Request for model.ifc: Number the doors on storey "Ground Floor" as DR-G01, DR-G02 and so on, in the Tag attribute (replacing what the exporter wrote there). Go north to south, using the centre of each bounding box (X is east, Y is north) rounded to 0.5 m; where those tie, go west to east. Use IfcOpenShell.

First a look at what the model holds.

```python
import ifcopenshell
import ifcopenshell.util.element
import ifcopenshell.util.placement

model = ifcopenshell.open("model.ifc")
print(model.schema)
storey = next(s for s in model.by_type("IfcBuildingStorey") if s.Name == "Ground Floor")
doors = [e for e in ifcopenshell.util.element.get_decomposition(storey) if e.is_a("IfcDoor")]
for e in sorted(doors, key=lambda e: e.id()):
    origin = ifcopenshell.util.placement.get_local_placement(e.ObjectPlacement)[:3, 3]
    print(e.id(), e.Tag, e.Name, origin.round(2) + 0.0, sep=" | ")
```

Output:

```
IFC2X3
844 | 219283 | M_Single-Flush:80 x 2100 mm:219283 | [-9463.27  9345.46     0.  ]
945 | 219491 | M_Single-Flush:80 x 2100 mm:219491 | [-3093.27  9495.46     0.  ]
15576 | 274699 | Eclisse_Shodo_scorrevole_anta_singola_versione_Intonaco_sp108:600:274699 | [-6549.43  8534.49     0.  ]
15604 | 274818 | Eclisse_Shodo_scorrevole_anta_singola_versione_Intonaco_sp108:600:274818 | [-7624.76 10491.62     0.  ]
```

```python
import ifcopenshell
import ifcopenshell.geom
import ifcopenshell.util.element
import ifcopenshell.util.shape

model = ifcopenshell.open("model.ifc")
settings = ifcopenshell.geom.settings()
settings.set("use-world-coords", True)


def centre(element):
    shape = ifcopenshell.geom.create_shape(settings, element)
    return ifcopenshell.util.shape.get_bbox_centroid(shape.geometry)


storey = next(s for s in model.by_type("IfcBuildingStorey") if s.Name == "Ground Floor")
doors = [e for e in ifcopenshell.util.element.get_decomposition(storey) if e.is_a("IfcDoor")]

# Insertion points can sit at a corner or the storey origin, so sort by the geometry (in metres).
centres = {e: centre(e) for e in doors}
doors.sort(key=lambda e: (-round(centres[e][1] / 0.5), centres[e][0]))

for i, e in enumerate(doors, start=1):
    number = f"DR-G{i:02d}"
    e.Tag = number
    print(e.id(), number)

model.write("model_rev.ifc")
```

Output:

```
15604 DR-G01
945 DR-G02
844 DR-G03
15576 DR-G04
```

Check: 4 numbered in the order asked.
